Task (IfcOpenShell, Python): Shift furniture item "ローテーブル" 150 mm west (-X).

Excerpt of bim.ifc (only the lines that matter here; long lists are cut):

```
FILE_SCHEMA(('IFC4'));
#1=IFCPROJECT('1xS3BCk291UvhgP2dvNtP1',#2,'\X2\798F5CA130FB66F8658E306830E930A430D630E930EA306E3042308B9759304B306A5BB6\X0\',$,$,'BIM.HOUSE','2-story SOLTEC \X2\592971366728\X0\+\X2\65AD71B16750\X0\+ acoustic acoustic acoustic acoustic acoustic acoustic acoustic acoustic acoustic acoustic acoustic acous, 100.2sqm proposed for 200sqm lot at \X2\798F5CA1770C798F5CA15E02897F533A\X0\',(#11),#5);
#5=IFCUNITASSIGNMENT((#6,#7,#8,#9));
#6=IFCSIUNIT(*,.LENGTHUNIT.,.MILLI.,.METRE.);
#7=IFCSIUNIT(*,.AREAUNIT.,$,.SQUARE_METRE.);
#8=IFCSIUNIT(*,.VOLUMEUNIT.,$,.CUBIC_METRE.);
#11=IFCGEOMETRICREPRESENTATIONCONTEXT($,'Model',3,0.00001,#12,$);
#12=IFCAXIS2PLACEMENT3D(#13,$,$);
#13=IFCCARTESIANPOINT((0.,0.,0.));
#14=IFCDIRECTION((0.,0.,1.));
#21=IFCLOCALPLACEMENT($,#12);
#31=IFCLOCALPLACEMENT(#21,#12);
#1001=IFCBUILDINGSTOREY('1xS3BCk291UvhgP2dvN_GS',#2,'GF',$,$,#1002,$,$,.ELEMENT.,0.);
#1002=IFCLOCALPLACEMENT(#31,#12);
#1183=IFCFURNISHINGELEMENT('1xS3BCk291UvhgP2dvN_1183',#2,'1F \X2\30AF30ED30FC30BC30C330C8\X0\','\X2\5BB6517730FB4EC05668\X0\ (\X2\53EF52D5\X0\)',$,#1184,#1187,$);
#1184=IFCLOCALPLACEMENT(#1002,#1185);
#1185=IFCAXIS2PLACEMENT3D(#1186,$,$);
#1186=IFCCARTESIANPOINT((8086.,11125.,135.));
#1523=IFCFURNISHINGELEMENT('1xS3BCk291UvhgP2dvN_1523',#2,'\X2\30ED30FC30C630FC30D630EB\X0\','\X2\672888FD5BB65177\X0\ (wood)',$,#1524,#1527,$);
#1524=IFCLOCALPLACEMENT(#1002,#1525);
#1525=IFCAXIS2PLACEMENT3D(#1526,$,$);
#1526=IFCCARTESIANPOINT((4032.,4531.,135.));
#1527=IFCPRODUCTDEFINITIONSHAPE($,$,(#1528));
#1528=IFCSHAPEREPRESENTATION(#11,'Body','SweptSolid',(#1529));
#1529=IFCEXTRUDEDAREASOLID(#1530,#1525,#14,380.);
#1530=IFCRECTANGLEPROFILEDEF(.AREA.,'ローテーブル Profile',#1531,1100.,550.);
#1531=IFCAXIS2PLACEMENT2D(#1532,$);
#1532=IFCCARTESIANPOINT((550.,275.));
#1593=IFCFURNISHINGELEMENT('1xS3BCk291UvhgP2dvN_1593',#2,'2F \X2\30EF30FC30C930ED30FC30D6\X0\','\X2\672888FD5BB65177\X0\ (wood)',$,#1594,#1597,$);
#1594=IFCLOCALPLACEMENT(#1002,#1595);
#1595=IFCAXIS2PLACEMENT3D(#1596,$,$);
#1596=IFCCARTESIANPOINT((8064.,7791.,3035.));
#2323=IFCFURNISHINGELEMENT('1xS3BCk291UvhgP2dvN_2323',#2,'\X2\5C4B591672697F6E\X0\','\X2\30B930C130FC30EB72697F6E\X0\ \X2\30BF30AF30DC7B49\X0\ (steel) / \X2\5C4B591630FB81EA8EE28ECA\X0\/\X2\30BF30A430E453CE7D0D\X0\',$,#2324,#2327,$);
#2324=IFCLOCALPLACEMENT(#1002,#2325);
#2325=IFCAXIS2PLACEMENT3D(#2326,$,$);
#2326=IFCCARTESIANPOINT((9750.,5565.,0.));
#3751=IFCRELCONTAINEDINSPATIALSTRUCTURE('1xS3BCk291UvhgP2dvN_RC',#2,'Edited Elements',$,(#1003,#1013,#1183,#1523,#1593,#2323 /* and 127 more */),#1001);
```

```python
import ifcopenshell
import ifcopenshell.api.geometry
import ifcopenshell.util.placement

model = ifcopenshell.open("bim.ifc")

item = model.by_guid("1xS3BCk291UvhgP2dvN_1523")
matrix = ifcopenshell.util.placement.get_local_placement(item.ObjectPlacement)
matrix[0, 3] -= 150.0
ifcopenshell.api.geometry.edit_object_placement(model, product=item, matrix=matrix, is_si=False)

print(ifcopenshell.util.placement.get_local_placement(item.ObjectPlacement).round(3) + 0.0)

model.write("bim_rev.ifc")
```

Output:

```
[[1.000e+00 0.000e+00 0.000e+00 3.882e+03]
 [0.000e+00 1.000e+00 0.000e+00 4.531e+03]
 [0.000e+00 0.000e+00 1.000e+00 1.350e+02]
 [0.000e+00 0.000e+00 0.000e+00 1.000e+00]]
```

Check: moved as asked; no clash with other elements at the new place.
